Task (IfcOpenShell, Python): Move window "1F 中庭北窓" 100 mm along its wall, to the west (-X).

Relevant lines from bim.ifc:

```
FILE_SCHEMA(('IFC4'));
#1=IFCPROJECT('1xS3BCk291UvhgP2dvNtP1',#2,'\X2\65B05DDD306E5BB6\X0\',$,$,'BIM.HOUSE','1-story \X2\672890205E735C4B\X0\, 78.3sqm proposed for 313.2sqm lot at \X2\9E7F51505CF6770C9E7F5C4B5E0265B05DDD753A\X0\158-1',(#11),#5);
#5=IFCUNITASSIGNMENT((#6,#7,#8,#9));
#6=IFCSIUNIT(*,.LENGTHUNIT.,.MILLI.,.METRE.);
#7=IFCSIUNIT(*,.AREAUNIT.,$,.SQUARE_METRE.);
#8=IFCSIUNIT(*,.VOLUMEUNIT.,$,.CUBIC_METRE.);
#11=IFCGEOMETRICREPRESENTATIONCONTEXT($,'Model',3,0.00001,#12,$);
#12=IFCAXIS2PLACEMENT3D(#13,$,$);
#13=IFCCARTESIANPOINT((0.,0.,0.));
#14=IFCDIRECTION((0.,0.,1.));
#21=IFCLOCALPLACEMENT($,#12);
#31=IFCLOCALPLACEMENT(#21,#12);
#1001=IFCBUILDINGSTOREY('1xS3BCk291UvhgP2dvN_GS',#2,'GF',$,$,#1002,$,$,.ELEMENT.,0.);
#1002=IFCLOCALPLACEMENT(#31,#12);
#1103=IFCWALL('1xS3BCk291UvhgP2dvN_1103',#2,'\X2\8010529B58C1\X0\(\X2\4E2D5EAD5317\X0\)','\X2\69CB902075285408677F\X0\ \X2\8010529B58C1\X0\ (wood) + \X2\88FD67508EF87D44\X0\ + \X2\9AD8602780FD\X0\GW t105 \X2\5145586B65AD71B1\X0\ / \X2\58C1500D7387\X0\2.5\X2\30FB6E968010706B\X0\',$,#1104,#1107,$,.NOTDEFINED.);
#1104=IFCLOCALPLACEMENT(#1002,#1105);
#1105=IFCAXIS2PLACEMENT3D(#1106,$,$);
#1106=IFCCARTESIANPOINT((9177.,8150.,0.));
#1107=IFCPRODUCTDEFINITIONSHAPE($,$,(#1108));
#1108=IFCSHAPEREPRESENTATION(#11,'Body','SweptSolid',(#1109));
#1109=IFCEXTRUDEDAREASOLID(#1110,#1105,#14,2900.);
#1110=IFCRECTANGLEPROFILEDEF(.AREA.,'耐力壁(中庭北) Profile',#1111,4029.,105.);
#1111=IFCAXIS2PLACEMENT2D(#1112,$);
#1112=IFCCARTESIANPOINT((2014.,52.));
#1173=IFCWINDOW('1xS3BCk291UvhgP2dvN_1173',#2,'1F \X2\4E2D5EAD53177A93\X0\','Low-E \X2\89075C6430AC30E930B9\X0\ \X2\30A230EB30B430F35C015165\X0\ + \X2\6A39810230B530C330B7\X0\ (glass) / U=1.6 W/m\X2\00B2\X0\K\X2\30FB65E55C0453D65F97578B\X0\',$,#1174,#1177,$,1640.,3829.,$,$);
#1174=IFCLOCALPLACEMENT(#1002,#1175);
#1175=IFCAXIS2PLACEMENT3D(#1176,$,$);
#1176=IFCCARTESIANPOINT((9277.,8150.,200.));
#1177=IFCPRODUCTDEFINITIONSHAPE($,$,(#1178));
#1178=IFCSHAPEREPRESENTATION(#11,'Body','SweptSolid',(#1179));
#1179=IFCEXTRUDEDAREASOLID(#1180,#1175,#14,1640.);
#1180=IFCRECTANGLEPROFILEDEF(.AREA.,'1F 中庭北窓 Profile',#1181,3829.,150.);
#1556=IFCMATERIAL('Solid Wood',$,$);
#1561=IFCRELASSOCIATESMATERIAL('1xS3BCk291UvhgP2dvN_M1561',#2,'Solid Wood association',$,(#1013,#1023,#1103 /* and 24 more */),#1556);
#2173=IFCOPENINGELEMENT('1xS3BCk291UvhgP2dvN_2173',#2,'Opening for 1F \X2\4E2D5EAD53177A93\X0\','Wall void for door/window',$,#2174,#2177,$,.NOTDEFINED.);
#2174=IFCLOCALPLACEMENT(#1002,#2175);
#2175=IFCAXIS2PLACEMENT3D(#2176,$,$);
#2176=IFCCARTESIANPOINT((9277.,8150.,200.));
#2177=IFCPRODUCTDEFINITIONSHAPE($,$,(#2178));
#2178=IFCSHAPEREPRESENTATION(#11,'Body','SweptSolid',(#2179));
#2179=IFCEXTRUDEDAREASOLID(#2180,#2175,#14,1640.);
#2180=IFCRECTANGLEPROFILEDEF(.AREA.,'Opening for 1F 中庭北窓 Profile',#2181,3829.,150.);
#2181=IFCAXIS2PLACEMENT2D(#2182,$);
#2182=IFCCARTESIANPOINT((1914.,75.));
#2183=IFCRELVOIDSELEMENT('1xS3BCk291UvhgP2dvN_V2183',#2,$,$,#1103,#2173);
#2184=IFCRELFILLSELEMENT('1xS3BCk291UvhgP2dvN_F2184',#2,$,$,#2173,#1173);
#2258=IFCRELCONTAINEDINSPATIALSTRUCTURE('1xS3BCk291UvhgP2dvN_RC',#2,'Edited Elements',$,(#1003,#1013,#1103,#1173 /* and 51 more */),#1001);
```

```python
import ifcopenshell
import ifcopenshell.api.geometry
import ifcopenshell.util.placement

model = ifcopenshell.open("bim.ifc")

window = model.by_id(1173)
opening = window.FillsVoids[0].RelatingOpeningElement
wall = opening.VoidsElements[0].RelatingBuildingElement

wall_matrix = ifcopenshell.util.placement.get_local_placement(wall.ObjectPlacement)
shift = wall_matrix[:3, 0] * -100.0
before = ifcopenshell.util.placement.get_local_placement(window.ObjectPlacement)[:3, 3].copy()

# The window is not placed relative to its opening, so move both.
for product in (opening, window):
    matrix = ifcopenshell.util.placement.get_local_placement(product.ObjectPlacement)
    matrix[:3, 3] += shift
    ifcopenshell.api.geometry.edit_object_placement(model, product=product, matrix=matrix, is_si=False)

after = ifcopenshell.util.placement.get_local_placement(window.ObjectPlacement)[:3, 3]
print("window moved by", (after - before).round(3) + 0.0)

model.write("bim_updated.ifc")
```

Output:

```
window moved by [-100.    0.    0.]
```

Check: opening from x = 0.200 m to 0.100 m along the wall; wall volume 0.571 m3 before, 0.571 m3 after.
